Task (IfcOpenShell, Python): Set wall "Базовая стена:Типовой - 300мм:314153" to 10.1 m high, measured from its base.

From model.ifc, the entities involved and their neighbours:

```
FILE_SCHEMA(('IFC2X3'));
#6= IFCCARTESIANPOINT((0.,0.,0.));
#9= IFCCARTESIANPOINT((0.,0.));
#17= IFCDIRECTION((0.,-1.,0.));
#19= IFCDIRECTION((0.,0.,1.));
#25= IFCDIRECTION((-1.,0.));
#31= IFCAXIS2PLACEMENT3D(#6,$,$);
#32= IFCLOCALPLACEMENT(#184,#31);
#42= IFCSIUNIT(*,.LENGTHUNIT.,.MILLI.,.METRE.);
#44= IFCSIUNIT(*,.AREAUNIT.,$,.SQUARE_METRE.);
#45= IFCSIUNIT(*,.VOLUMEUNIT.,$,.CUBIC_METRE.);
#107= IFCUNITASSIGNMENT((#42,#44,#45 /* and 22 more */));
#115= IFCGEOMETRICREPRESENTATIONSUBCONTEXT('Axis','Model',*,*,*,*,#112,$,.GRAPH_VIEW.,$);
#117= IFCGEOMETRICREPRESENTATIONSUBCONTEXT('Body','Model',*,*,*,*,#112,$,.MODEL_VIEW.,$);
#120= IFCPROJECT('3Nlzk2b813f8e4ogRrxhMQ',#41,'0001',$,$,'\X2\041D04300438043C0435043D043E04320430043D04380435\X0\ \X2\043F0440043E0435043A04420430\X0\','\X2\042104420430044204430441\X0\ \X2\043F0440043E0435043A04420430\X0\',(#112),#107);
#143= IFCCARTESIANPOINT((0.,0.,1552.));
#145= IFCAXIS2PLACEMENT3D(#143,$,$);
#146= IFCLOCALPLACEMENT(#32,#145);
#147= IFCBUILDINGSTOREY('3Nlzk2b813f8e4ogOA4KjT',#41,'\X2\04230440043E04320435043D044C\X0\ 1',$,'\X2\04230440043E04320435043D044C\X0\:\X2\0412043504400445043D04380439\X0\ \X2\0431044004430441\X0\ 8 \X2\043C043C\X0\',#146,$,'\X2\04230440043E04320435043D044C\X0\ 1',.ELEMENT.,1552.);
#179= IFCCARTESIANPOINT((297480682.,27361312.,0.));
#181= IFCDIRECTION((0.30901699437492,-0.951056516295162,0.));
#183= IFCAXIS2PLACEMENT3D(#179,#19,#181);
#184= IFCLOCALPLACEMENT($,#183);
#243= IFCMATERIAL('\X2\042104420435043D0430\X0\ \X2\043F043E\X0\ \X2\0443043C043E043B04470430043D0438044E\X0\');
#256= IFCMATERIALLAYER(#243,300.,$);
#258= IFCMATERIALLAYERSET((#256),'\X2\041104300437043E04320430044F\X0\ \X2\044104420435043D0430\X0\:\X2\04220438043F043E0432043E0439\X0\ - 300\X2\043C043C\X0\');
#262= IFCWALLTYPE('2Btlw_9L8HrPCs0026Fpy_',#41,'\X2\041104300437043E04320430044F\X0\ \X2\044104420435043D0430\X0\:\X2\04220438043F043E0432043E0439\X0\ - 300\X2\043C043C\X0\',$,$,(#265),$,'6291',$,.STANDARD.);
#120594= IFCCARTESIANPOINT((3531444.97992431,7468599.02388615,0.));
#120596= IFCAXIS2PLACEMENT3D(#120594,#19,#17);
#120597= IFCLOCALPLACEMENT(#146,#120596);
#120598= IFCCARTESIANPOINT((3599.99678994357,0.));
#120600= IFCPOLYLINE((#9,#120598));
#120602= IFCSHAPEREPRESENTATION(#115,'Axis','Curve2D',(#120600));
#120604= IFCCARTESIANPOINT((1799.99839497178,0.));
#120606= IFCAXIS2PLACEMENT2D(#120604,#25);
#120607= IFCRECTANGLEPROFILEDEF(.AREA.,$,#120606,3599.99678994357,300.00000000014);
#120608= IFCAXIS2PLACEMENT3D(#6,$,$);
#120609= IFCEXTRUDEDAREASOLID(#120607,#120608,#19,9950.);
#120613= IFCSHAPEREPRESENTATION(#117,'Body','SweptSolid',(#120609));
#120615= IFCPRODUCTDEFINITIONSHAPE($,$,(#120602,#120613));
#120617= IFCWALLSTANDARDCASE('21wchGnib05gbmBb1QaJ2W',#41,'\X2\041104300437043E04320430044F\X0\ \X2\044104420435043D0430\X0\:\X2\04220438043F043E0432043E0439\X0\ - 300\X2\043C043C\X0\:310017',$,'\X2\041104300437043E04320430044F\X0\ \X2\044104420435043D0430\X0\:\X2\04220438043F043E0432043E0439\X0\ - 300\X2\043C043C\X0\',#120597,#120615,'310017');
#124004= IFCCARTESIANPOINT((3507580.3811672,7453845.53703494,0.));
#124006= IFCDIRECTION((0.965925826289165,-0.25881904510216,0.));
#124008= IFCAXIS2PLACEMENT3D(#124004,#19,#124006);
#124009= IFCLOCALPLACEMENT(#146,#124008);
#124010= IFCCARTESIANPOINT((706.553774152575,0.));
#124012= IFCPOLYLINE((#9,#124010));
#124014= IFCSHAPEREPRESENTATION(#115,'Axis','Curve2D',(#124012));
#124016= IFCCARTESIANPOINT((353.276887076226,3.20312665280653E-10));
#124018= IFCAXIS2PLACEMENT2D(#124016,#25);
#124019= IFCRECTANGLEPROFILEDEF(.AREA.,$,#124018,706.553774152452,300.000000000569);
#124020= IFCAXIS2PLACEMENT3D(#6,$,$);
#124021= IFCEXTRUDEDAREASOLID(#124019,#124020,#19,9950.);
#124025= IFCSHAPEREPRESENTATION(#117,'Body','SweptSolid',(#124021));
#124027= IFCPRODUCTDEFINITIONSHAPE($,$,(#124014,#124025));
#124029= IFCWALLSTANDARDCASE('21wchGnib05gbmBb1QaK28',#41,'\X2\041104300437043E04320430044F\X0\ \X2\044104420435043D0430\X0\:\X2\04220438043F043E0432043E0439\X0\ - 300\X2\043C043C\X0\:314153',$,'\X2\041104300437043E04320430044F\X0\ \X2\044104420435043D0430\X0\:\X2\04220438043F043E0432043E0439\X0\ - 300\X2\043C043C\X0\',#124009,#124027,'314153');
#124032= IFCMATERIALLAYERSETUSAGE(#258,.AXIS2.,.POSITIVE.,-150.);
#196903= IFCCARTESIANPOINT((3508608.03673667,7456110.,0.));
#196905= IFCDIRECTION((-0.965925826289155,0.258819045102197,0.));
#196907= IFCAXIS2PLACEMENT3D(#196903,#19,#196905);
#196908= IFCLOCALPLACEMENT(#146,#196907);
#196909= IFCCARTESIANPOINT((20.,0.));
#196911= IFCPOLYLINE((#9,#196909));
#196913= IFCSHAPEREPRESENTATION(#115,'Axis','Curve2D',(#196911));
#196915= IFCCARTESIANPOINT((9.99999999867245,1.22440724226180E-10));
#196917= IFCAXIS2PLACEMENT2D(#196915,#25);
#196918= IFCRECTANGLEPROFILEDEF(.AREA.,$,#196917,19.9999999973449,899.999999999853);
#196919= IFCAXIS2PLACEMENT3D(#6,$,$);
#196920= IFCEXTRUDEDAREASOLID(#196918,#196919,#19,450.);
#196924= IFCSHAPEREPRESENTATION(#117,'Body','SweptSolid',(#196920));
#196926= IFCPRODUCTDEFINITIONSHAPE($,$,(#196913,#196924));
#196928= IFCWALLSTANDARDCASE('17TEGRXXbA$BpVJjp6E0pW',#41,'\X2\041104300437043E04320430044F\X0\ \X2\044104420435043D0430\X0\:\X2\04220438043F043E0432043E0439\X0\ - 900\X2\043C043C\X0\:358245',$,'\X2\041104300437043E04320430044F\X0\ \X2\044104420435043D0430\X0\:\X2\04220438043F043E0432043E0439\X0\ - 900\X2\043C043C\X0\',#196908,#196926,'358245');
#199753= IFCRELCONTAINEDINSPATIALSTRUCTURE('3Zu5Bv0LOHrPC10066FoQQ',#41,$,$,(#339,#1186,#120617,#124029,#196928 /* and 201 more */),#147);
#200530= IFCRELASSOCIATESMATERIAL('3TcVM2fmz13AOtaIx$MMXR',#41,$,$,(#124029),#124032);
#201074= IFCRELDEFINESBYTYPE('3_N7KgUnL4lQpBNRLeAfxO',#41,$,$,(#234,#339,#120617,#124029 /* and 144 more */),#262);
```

```python
import ifcopenshell
import ifcopenshell.geom
import ifcopenshell.util.representation
import ifcopenshell.util.shape
import ifcopenshell.util.unit

model = ifcopenshell.open("model.ifc")
unit_scale = ifcopenshell.util.unit.calculate_unit_scale(model)
settings = ifcopenshell.geom.settings()


def volume(element):
    """Net volume in cubic metres, openings subtracted."""
    shape = ifcopenshell.geom.create_shape(settings, element)
    return ifcopenshell.util.shape.get_volume(shape.geometry)


wall = model.by_id(124029)
before = volume(wall)

body = ifcopenshell.util.representation.get_representation(wall, "Model", "Body")
solid = body.Items[0]
old_height = solid.Depth
solid.Depth = 10.1 / unit_scale
after = volume(wall)

print(f"height {old_height:g} -> {solid.Depth:g}, volume {before:.3f} -> {after:.3f} m3")

model.write("model-out.ifc")
```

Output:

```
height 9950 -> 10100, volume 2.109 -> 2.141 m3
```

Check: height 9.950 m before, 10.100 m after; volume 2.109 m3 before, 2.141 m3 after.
